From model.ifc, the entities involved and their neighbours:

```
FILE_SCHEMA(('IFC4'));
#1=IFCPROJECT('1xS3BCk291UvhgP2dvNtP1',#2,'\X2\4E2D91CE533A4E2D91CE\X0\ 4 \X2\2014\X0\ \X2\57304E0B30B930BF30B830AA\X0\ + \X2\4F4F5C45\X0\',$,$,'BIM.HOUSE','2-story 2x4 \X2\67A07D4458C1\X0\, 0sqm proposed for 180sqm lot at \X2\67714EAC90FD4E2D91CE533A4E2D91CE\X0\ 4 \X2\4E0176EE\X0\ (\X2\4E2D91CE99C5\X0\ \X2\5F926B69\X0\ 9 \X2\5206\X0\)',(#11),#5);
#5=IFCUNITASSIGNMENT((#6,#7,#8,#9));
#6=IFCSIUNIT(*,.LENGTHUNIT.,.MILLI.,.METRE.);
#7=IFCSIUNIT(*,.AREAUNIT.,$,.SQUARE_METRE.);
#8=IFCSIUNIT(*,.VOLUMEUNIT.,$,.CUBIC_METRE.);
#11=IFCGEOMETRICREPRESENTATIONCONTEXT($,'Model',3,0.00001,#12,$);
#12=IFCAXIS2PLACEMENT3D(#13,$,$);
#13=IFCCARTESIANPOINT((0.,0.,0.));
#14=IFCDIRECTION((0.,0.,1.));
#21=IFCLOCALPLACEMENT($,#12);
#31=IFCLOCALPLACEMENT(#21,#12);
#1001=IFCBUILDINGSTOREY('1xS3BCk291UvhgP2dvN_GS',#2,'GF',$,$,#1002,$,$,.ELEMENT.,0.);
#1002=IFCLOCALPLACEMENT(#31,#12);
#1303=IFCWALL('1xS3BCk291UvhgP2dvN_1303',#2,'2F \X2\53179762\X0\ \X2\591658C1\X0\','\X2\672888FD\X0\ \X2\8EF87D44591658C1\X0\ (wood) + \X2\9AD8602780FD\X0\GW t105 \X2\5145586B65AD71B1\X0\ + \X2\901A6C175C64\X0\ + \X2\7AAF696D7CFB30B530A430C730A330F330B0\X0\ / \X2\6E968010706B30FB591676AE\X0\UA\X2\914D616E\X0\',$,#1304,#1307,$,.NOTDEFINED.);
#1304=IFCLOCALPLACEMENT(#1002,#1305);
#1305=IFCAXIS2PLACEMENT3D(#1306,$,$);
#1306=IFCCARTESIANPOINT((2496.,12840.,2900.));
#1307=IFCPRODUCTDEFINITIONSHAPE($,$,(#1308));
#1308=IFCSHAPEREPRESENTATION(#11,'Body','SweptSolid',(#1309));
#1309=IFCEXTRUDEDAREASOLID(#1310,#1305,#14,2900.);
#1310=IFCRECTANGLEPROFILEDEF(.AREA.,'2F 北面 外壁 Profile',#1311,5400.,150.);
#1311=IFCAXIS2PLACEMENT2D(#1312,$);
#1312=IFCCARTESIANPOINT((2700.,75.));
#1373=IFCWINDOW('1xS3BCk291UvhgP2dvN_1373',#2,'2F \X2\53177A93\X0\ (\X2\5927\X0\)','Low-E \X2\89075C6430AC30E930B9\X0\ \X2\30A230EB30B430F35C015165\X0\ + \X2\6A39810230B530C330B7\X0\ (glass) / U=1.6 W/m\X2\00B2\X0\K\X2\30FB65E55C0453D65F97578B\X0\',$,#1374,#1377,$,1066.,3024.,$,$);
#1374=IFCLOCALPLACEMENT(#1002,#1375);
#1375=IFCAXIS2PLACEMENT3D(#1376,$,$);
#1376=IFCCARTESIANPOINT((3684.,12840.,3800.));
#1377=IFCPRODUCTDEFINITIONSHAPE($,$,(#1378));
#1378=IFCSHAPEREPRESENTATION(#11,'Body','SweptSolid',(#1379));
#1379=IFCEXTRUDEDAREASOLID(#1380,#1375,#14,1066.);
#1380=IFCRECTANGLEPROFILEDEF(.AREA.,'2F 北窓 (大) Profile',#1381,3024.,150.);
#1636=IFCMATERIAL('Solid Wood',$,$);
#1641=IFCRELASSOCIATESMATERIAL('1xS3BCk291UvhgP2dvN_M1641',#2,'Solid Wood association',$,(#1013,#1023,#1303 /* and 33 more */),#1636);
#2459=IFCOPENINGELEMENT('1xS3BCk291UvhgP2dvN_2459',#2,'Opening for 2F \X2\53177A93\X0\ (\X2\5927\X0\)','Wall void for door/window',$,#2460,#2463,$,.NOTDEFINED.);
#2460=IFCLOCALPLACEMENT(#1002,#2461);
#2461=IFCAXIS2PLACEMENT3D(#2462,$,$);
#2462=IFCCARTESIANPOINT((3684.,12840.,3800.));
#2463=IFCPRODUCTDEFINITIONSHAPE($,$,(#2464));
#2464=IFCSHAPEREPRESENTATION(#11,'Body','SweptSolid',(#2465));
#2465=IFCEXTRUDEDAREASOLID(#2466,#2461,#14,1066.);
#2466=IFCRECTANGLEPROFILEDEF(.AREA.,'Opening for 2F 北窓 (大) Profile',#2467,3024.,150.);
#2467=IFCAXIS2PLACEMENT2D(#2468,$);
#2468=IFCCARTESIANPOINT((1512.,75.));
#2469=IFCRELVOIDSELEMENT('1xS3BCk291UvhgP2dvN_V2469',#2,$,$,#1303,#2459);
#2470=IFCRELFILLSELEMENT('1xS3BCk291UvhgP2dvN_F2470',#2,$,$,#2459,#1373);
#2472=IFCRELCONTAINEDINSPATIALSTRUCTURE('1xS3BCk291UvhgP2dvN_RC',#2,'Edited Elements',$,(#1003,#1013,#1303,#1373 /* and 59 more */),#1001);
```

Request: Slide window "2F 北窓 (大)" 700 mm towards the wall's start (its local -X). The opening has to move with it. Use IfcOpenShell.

```python
import ifcopenshell
import ifcopenshell.api.geometry
import ifcopenshell.util.placement

model = ifcopenshell.open("model.ifc")

window = model.by_guid("1xS3BCk291UvhgP2dvN_1373")
opening = window.FillsVoids[0].RelatingOpeningElement
wall = opening.VoidsElements[0].RelatingBuildingElement

wall_matrix = ifcopenshell.util.placement.get_local_placement(wall.ObjectPlacement)
shift = wall_matrix[:3, 0] * -700.0
before = ifcopenshell.util.placement.get_local_placement(window.ObjectPlacement)[:3, 3].copy()

# The window is not placed relative to its opening, so move both.
for product in (opening, window):
    matrix = ifcopenshell.util.placement.get_local_placement(product.ObjectPlacement)
    matrix[:3, 3] += shift
    ifcopenshell.api.geometry.edit_object_placement(model, product=product, matrix=matrix, is_si=False)

after = ifcopenshell.util.placement.get_local_placement(window.ObjectPlacement)[:3, 3]
print("window moved by", (after - before).round(3) + 0.0)

model.write("model_v2.ifc")
```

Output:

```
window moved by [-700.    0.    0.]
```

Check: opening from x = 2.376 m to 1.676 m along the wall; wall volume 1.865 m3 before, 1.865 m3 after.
